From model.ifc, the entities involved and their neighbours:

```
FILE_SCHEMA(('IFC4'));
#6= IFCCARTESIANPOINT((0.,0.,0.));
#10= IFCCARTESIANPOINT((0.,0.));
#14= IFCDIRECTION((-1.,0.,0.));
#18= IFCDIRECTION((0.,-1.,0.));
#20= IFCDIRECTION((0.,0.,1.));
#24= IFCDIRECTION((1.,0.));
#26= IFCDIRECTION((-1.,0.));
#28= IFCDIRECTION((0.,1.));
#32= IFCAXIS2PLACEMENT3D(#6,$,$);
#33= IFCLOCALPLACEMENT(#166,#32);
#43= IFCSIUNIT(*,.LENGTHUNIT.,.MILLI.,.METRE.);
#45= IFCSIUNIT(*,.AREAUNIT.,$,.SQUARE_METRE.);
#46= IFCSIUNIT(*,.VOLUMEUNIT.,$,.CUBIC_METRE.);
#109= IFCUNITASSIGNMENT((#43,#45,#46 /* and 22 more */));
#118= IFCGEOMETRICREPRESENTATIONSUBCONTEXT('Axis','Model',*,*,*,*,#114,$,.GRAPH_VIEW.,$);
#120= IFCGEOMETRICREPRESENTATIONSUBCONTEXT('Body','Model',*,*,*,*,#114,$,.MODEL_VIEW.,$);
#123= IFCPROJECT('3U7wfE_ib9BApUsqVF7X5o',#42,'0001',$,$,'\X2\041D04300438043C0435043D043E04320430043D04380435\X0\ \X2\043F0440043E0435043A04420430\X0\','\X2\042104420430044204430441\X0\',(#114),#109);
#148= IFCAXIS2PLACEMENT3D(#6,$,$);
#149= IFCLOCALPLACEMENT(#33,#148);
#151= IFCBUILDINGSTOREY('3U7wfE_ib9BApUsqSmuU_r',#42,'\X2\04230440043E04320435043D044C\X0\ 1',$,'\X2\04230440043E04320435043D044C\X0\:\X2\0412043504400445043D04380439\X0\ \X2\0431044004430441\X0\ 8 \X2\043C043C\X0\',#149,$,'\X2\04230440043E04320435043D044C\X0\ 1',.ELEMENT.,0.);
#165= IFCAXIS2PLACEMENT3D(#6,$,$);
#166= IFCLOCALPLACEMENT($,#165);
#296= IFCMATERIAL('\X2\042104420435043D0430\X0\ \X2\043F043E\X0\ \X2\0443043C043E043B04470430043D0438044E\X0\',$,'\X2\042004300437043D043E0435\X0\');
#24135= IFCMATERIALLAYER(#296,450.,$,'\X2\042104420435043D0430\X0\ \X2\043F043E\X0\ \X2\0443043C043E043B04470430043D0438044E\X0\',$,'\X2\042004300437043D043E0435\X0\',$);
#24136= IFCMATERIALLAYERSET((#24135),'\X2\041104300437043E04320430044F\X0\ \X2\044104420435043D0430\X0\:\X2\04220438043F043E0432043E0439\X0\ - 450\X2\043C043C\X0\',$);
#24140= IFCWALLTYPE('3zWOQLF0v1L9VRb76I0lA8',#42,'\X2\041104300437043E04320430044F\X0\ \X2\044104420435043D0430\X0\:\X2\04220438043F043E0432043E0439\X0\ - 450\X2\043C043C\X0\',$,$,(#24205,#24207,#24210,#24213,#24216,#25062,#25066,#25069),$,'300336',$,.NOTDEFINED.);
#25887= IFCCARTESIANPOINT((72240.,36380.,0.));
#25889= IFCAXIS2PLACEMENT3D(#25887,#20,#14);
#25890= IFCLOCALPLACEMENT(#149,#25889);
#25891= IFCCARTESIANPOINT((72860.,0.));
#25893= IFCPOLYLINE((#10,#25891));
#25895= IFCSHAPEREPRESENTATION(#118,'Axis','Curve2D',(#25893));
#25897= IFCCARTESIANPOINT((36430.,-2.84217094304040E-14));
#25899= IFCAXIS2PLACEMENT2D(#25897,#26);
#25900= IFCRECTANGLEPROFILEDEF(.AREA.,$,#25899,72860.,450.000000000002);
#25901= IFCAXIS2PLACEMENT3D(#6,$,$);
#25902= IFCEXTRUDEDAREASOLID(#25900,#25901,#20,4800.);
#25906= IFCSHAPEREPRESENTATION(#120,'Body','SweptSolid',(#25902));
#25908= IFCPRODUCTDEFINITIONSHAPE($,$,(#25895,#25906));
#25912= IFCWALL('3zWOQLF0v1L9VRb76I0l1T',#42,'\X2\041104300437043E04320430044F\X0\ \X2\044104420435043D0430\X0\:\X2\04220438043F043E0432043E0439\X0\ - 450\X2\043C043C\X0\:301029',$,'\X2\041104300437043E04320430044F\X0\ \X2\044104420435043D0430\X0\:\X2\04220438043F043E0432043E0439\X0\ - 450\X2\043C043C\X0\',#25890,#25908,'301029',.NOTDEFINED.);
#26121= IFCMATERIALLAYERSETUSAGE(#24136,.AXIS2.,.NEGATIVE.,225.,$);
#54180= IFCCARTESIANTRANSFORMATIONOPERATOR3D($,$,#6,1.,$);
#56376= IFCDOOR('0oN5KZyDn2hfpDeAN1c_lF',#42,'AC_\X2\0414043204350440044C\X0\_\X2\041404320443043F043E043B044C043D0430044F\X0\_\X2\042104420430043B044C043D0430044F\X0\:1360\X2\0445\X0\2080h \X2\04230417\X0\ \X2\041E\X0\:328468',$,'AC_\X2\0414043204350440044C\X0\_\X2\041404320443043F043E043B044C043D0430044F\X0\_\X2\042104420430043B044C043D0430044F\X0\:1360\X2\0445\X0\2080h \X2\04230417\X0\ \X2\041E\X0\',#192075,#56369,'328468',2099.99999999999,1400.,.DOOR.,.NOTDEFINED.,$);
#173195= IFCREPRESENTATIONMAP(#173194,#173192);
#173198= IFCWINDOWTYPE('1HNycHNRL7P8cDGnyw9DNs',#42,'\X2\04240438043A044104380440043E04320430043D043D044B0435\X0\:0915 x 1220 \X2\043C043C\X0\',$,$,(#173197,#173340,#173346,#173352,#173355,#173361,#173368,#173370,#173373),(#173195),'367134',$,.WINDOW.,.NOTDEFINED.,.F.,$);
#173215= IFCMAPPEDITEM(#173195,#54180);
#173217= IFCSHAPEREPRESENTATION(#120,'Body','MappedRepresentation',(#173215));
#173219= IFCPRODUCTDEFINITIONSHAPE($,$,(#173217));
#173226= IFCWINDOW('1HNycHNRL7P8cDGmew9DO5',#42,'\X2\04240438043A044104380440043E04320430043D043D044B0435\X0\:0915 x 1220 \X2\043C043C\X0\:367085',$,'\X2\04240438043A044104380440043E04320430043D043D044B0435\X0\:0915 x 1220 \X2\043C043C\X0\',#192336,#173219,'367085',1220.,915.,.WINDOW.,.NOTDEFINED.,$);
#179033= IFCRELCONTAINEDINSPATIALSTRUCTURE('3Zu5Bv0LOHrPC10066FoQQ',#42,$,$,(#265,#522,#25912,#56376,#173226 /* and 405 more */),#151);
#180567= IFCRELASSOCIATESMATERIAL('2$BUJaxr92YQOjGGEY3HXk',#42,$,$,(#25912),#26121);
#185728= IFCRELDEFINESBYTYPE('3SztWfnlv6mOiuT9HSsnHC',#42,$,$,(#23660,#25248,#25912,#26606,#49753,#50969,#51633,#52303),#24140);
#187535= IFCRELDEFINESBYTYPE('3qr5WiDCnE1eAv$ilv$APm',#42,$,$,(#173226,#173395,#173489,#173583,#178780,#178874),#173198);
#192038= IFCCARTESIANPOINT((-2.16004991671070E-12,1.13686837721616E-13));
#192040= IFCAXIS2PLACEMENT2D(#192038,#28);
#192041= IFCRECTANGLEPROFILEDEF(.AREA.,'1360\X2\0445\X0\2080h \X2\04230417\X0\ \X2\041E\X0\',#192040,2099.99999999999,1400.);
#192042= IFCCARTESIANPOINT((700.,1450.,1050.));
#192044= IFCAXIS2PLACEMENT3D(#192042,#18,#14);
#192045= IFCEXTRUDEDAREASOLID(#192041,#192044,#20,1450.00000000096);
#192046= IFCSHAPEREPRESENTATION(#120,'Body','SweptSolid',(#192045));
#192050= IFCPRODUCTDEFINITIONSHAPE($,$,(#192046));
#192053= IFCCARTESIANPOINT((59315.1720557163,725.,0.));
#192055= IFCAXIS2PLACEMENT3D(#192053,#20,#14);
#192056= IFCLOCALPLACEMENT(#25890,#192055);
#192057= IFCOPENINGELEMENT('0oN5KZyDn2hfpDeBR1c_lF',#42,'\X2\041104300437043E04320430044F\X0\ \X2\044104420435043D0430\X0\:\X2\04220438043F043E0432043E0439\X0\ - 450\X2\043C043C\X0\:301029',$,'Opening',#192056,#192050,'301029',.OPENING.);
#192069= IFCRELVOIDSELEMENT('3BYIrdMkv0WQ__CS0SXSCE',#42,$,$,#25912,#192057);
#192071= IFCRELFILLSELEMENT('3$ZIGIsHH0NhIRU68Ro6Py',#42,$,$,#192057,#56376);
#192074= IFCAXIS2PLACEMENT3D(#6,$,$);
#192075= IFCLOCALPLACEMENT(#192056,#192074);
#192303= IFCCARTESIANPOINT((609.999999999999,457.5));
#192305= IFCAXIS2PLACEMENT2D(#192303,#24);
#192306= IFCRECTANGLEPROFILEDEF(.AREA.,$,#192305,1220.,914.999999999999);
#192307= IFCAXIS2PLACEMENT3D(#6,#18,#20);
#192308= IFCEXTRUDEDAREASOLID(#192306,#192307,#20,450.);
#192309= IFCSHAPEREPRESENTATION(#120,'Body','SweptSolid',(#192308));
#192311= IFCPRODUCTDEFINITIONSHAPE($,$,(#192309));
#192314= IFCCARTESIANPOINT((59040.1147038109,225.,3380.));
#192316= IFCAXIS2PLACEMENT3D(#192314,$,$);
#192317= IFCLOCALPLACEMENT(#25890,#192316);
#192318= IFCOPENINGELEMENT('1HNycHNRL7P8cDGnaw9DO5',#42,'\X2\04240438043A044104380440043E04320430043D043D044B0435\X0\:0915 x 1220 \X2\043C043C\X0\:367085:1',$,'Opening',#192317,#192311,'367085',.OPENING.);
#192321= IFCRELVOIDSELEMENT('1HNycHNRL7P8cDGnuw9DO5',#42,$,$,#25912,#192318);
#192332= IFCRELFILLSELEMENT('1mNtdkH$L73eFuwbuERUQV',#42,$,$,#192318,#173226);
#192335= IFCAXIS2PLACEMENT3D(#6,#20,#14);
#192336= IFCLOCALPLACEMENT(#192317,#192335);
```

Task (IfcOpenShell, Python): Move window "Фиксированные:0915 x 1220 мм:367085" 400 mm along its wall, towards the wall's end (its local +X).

```python
import ifcopenshell
import ifcopenshell.api.geometry
import ifcopenshell.util.placement
import ifcopenshell.util.unit

model = ifcopenshell.open("model.ifc")
unit_scale = ifcopenshell.util.unit.calculate_unit_scale(model)

window = model.by_guid("1HNycHNRL7P8cDGmew9DO5")
opening = window.FillsVoids[0].RelatingOpeningElement
wall = opening.VoidsElements[0].RelatingBuildingElement

wall_matrix = ifcopenshell.util.placement.get_local_placement(wall.ObjectPlacement)
shift = wall_matrix[:3, 0] * 0.4 / unit_scale
before = ifcopenshell.util.placement.get_local_placement(window.ObjectPlacement)[:3, 3].copy()

# The window is placed relative to its opening, so it follows when the opening moves.
matrix = ifcopenshell.util.placement.get_local_placement(opening.ObjectPlacement)
matrix[:3, 3] += shift
ifcopenshell.api.geometry.edit_object_placement(
    model, product=opening, matrix=matrix, is_si=False, should_transform_children=True
)

after = ifcopenshell.util.placement.get_local_placement(window.ObjectPlacement)[:3, 3]
print("window moved by", (after - before).round(3) + 0.0)

model.write("model-out.ifc")
```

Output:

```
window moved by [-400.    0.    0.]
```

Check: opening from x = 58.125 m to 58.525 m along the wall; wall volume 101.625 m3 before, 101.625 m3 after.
